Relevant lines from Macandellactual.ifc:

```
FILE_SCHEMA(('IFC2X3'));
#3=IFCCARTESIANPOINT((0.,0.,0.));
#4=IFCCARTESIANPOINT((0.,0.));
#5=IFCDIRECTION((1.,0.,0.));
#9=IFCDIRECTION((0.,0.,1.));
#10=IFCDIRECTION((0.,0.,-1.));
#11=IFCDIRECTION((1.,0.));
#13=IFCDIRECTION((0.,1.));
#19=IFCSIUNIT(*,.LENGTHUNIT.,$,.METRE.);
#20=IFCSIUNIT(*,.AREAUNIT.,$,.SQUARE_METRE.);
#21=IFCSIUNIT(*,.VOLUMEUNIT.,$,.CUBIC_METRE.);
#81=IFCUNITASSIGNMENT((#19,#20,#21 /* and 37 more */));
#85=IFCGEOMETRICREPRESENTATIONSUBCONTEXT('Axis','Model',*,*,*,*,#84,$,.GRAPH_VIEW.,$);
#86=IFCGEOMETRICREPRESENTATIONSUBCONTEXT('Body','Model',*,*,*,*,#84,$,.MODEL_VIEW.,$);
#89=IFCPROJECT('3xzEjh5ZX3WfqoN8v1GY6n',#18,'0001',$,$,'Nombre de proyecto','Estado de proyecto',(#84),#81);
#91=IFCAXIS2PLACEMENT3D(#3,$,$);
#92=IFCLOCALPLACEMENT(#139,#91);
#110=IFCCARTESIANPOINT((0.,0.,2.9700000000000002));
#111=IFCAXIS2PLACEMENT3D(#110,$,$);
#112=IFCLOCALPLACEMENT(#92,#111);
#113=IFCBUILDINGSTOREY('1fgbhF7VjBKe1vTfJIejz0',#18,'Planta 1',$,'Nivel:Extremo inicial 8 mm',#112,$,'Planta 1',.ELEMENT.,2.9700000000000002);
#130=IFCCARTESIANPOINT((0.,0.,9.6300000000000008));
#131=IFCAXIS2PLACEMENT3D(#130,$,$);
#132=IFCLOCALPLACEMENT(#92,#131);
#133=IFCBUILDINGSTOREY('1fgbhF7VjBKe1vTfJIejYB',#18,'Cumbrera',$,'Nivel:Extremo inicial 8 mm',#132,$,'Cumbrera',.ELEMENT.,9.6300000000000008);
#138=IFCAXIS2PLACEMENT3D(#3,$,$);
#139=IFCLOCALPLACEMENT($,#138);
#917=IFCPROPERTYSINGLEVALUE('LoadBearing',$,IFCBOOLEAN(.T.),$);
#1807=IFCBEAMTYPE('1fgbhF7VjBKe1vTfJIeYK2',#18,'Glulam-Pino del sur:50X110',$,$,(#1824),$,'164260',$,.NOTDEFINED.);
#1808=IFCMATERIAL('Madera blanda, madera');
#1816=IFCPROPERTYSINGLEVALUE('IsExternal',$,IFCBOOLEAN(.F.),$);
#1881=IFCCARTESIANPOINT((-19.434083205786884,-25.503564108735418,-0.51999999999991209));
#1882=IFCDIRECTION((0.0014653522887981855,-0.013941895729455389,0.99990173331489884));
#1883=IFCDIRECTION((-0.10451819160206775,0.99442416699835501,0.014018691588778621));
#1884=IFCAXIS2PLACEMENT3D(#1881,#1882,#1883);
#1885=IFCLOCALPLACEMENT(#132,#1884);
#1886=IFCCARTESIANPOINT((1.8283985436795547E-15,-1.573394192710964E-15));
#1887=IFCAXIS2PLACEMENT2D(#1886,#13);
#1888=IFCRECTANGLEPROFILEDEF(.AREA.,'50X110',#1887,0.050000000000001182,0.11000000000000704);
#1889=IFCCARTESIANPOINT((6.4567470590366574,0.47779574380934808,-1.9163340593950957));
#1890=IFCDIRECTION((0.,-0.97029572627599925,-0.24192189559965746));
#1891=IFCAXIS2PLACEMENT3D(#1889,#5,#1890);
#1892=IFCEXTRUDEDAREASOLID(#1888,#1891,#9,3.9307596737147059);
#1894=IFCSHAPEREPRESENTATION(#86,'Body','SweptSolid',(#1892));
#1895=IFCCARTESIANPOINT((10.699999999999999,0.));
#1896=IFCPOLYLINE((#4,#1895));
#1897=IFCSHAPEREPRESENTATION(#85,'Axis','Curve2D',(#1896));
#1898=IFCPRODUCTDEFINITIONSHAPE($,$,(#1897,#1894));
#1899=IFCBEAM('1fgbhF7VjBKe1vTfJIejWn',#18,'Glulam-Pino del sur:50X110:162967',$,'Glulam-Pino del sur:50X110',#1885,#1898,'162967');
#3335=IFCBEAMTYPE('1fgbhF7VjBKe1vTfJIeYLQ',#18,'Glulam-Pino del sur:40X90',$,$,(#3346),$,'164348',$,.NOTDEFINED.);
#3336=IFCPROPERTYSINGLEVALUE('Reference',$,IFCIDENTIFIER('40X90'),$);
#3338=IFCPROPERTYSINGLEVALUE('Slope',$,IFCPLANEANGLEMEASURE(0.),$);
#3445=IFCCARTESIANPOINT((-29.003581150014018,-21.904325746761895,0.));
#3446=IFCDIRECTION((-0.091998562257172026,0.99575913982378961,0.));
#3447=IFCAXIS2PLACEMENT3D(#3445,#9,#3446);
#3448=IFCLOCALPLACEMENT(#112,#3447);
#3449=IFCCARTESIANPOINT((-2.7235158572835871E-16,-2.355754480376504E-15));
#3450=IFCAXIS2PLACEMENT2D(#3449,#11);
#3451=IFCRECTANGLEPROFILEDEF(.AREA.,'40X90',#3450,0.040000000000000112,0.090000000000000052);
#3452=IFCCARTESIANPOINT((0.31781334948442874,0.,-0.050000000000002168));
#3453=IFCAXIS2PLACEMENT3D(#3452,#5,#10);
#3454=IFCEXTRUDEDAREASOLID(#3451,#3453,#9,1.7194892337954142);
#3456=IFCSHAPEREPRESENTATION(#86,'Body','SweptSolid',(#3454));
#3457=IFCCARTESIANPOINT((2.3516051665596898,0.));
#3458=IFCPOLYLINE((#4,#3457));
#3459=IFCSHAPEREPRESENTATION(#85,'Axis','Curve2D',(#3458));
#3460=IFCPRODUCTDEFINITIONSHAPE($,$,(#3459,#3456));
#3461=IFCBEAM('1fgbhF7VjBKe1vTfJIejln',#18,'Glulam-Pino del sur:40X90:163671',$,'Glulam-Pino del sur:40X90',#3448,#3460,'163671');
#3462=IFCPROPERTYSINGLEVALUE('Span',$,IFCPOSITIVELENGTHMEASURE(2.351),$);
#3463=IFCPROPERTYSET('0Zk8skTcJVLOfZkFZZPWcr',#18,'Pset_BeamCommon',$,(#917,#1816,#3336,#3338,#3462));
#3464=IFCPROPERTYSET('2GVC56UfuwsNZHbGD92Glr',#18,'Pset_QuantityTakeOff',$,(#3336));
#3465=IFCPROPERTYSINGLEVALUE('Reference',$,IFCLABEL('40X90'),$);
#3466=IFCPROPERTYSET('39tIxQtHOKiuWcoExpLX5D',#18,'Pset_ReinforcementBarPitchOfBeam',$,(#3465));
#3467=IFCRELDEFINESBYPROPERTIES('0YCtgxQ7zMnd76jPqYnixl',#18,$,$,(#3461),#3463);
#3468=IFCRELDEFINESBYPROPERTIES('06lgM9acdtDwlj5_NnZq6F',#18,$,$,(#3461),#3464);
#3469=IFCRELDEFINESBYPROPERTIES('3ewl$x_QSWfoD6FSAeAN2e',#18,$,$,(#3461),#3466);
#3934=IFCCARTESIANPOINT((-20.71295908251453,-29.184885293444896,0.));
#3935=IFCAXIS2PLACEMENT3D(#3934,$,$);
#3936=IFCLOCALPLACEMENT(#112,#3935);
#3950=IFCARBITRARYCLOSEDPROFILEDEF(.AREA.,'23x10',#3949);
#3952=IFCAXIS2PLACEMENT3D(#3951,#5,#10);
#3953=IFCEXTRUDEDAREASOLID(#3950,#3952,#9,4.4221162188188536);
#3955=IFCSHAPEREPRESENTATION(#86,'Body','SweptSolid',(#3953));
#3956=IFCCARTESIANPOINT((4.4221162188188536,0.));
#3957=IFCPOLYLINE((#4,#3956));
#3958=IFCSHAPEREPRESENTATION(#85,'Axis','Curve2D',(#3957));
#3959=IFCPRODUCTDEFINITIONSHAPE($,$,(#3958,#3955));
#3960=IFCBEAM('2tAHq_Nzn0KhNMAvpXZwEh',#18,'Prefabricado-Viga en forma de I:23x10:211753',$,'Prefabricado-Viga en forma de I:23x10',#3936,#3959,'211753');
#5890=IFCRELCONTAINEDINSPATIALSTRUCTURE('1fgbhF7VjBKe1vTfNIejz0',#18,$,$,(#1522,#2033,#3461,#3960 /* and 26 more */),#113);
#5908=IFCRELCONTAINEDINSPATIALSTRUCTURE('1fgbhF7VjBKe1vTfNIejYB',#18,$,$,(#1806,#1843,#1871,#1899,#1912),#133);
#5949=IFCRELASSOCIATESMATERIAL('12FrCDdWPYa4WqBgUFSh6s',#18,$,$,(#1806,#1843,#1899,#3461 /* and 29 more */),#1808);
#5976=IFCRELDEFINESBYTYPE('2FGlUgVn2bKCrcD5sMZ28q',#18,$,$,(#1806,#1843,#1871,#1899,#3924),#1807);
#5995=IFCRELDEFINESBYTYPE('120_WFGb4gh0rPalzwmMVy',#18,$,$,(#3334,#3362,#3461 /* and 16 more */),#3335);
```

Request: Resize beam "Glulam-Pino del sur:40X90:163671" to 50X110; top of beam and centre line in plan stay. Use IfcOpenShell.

```python
import ifcopenshell
import ifcopenshell.api.pset
import ifcopenshell.api.type
import ifcopenshell.util.element
import ifcopenshell.util.representation

model = ifcopenshell.open("Macandellactual.ifc")

member = model.by_id(3461)
source = next(p for p in model.by_type("IfcRectangleProfileDef") if p.ProfileName == "50X110")

body = ifcopenshell.util.representation.get_representation(member, "Model", "Body")
solid = body.Items[0]
old_profile = solid.SweptArea

# Copy the section's sizes but keep this member's own profile position.
profile = ifcopenshell.util.element.copy(model, source)
# Profiles are centred, so shift by half the change in depth to hold the top.
shift = (old_profile.XDim - profile.XDim) / 2
x, y = old_profile.Position.Location.Coordinates
up = (-1.0, 0.0)  # upwards, in the solid's own plane
location = model.createIfcCartesianPoint((x + up[0] * shift, y + up[1] * shift))
profile.Position = model.createIfcAxis2Placement2D(location, old_profile.Position.RefDirection)
solid.SweptArea = profile
if not model.get_total_inverses(old_profile):
    ifcopenshell.util.element.remove_deep2(model, old_profile)

new_type = model.by_id(1807)
ifcopenshell.api.type.assign_type(
    model, related_objects=[member], relating_type=new_type, should_map_representations=False
)
member.Name = member.Name.replace("40X90", "50X110")
member.ObjectType = "Glulam-Pino del sur:50X110"
pset = model.by_id(ifcopenshell.util.element.get_pset(member, "Pset_BeamCommon", should_inherit=False)["id"])
ifcopenshell.api.pset.edit_pset(model, pset=pset, properties={"Reference": "50X110"})
pset = model.by_id(ifcopenshell.util.element.get_pset(member, "Pset_QuantityTakeOff", should_inherit=False)["id"])
ifcopenshell.api.pset.edit_pset(model, pset=pset, properties={"Reference": "50X110"})
pset = model.by_id(ifcopenshell.util.element.get_pset(member, "Pset_ReinforcementBarPitchOfBeam", should_inherit=False)["id"])
ifcopenshell.api.pset.edit_pset(model, pset=pset, properties={"Reference": "50X110"})

print(solid.SweptArea)

model.write("Macandellactual-out.ifc")
```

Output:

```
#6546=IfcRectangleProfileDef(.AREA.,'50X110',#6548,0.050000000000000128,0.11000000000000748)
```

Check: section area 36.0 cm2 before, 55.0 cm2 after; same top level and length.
